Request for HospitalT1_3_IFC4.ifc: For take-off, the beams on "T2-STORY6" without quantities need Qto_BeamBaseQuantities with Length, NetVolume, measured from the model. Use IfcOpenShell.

First a look at what the model holds.

```python
import ifcopenshell
import ifcopenshell.util.element
import ifcopenshell.util.unit

model = ifcopenshell.open("HospitalT1_3_IFC4.ifc")
print(model.schema)
for unit_type in ("LENGTHUNIT", "AREAUNIT", "VOLUMEUNIT"):
    print(unit_type, ifcopenshell.util.unit.calculate_unit_scale(model, unit_type))
storey = next(s for s in model.by_type("IfcBuildingStorey") if s.Name == "T2-STORY6")
beams = [e for e in ifcopenshell.util.element.get_decomposition(storey) if e.is_a("IfcBeam")]
for e in sorted(beams, key=lambda e: e.id()):
    print(e.id(), e.is_a(), e.Name, list(ifcopenshell.util.element.get_psets(e, qtos_only=True)), sep=" | ")
```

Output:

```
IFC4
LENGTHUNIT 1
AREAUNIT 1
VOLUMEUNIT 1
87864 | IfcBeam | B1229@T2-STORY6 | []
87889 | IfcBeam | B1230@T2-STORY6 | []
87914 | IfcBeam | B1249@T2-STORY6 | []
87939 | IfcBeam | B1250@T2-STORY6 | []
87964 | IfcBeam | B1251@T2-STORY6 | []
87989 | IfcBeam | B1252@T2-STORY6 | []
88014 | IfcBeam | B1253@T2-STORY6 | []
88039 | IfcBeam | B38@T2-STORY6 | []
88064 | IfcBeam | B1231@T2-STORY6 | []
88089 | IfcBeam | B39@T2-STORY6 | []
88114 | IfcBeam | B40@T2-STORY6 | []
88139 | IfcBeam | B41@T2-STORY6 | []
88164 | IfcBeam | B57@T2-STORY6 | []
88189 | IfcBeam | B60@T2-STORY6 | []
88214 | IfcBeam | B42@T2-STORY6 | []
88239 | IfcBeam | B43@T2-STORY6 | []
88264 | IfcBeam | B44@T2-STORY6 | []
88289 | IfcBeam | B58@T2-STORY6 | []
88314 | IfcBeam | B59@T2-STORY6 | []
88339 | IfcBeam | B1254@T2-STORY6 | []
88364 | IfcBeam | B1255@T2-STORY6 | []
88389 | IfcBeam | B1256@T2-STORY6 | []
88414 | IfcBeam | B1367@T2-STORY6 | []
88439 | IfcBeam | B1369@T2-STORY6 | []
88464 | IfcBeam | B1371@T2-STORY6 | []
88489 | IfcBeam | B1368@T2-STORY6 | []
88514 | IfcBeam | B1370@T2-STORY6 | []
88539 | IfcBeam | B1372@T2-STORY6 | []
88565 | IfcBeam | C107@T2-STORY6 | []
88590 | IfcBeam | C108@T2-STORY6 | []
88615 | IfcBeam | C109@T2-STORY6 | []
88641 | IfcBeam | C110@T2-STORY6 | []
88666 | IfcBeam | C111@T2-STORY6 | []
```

```python
import ifcopenshell
import ifcopenshell.api.pset
import ifcopenshell.geom
import ifcopenshell.util.element
import ifcopenshell.util.shape
import ifcopenshell.util.unit

model = ifcopenshell.open("HospitalT1_3_IFC4.ifc")
unit_scale = ifcopenshell.util.unit.calculate_unit_scale(model)
volume_scale = ifcopenshell.util.unit.calculate_unit_scale(model, "VOLUMEUNIT")
settings = ifcopenshell.geom.settings()

storey = next(s for s in model.by_type("IfcBuildingStorey") if s.Name == "T2-STORY6")
beams = [e for e in ifcopenshell.util.element.get_decomposition(storey) if e.is_a("IfcBeam")]

for e in sorted(beams, key=lambda e: e.id()):
    if ifcopenshell.util.element.get_psets(e, qtos_only=True, should_inherit=False):
        continue
    # Geometry comes back in metres, in the element's own axes.
    shape = ifcopenshell.geom.create_shape(settings, e)
    values = {
        "Length": ifcopenshell.util.shape.get_max_xyz(shape.geometry) / unit_scale,
        "NetVolume": ifcopenshell.util.shape.get_volume(shape.geometry) / volume_scale,
    }
    qto = ifcopenshell.api.pset.add_qto(model, product=e, name="Qto_BeamBaseQuantities")
    ifcopenshell.api.pset.edit_qto(model, qto=qto, properties=values)
    print(e.id(), {k: round(v, 3) for k, v in values.items()})

model.write("HospitalT1_3_IFC4_updated.ifc")
```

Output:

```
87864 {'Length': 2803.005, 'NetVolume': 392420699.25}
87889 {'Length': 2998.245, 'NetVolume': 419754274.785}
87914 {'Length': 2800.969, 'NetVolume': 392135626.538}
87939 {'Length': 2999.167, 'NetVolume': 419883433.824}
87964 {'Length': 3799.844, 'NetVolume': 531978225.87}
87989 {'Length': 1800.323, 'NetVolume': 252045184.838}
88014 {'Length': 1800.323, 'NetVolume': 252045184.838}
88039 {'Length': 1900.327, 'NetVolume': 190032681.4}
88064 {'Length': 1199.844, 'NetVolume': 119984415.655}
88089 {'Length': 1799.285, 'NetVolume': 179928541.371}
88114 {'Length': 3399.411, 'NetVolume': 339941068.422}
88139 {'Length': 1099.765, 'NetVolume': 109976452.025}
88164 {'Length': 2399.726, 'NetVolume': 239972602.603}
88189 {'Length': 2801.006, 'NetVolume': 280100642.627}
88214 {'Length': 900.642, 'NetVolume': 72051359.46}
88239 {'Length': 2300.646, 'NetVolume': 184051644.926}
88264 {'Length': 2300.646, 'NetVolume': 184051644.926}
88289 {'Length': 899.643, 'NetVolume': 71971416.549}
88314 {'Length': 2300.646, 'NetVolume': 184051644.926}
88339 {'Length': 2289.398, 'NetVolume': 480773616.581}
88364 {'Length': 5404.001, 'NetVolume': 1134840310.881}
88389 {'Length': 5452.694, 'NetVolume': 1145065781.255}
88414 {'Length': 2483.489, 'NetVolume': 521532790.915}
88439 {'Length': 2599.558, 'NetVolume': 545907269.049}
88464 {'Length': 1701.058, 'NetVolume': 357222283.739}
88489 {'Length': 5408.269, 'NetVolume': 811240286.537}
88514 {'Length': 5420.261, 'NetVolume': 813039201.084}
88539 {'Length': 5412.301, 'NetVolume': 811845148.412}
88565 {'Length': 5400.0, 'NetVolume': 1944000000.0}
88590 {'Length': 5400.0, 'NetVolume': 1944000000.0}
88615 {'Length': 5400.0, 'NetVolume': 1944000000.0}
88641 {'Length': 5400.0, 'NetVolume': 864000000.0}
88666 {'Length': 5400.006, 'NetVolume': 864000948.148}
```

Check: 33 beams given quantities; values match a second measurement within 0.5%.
